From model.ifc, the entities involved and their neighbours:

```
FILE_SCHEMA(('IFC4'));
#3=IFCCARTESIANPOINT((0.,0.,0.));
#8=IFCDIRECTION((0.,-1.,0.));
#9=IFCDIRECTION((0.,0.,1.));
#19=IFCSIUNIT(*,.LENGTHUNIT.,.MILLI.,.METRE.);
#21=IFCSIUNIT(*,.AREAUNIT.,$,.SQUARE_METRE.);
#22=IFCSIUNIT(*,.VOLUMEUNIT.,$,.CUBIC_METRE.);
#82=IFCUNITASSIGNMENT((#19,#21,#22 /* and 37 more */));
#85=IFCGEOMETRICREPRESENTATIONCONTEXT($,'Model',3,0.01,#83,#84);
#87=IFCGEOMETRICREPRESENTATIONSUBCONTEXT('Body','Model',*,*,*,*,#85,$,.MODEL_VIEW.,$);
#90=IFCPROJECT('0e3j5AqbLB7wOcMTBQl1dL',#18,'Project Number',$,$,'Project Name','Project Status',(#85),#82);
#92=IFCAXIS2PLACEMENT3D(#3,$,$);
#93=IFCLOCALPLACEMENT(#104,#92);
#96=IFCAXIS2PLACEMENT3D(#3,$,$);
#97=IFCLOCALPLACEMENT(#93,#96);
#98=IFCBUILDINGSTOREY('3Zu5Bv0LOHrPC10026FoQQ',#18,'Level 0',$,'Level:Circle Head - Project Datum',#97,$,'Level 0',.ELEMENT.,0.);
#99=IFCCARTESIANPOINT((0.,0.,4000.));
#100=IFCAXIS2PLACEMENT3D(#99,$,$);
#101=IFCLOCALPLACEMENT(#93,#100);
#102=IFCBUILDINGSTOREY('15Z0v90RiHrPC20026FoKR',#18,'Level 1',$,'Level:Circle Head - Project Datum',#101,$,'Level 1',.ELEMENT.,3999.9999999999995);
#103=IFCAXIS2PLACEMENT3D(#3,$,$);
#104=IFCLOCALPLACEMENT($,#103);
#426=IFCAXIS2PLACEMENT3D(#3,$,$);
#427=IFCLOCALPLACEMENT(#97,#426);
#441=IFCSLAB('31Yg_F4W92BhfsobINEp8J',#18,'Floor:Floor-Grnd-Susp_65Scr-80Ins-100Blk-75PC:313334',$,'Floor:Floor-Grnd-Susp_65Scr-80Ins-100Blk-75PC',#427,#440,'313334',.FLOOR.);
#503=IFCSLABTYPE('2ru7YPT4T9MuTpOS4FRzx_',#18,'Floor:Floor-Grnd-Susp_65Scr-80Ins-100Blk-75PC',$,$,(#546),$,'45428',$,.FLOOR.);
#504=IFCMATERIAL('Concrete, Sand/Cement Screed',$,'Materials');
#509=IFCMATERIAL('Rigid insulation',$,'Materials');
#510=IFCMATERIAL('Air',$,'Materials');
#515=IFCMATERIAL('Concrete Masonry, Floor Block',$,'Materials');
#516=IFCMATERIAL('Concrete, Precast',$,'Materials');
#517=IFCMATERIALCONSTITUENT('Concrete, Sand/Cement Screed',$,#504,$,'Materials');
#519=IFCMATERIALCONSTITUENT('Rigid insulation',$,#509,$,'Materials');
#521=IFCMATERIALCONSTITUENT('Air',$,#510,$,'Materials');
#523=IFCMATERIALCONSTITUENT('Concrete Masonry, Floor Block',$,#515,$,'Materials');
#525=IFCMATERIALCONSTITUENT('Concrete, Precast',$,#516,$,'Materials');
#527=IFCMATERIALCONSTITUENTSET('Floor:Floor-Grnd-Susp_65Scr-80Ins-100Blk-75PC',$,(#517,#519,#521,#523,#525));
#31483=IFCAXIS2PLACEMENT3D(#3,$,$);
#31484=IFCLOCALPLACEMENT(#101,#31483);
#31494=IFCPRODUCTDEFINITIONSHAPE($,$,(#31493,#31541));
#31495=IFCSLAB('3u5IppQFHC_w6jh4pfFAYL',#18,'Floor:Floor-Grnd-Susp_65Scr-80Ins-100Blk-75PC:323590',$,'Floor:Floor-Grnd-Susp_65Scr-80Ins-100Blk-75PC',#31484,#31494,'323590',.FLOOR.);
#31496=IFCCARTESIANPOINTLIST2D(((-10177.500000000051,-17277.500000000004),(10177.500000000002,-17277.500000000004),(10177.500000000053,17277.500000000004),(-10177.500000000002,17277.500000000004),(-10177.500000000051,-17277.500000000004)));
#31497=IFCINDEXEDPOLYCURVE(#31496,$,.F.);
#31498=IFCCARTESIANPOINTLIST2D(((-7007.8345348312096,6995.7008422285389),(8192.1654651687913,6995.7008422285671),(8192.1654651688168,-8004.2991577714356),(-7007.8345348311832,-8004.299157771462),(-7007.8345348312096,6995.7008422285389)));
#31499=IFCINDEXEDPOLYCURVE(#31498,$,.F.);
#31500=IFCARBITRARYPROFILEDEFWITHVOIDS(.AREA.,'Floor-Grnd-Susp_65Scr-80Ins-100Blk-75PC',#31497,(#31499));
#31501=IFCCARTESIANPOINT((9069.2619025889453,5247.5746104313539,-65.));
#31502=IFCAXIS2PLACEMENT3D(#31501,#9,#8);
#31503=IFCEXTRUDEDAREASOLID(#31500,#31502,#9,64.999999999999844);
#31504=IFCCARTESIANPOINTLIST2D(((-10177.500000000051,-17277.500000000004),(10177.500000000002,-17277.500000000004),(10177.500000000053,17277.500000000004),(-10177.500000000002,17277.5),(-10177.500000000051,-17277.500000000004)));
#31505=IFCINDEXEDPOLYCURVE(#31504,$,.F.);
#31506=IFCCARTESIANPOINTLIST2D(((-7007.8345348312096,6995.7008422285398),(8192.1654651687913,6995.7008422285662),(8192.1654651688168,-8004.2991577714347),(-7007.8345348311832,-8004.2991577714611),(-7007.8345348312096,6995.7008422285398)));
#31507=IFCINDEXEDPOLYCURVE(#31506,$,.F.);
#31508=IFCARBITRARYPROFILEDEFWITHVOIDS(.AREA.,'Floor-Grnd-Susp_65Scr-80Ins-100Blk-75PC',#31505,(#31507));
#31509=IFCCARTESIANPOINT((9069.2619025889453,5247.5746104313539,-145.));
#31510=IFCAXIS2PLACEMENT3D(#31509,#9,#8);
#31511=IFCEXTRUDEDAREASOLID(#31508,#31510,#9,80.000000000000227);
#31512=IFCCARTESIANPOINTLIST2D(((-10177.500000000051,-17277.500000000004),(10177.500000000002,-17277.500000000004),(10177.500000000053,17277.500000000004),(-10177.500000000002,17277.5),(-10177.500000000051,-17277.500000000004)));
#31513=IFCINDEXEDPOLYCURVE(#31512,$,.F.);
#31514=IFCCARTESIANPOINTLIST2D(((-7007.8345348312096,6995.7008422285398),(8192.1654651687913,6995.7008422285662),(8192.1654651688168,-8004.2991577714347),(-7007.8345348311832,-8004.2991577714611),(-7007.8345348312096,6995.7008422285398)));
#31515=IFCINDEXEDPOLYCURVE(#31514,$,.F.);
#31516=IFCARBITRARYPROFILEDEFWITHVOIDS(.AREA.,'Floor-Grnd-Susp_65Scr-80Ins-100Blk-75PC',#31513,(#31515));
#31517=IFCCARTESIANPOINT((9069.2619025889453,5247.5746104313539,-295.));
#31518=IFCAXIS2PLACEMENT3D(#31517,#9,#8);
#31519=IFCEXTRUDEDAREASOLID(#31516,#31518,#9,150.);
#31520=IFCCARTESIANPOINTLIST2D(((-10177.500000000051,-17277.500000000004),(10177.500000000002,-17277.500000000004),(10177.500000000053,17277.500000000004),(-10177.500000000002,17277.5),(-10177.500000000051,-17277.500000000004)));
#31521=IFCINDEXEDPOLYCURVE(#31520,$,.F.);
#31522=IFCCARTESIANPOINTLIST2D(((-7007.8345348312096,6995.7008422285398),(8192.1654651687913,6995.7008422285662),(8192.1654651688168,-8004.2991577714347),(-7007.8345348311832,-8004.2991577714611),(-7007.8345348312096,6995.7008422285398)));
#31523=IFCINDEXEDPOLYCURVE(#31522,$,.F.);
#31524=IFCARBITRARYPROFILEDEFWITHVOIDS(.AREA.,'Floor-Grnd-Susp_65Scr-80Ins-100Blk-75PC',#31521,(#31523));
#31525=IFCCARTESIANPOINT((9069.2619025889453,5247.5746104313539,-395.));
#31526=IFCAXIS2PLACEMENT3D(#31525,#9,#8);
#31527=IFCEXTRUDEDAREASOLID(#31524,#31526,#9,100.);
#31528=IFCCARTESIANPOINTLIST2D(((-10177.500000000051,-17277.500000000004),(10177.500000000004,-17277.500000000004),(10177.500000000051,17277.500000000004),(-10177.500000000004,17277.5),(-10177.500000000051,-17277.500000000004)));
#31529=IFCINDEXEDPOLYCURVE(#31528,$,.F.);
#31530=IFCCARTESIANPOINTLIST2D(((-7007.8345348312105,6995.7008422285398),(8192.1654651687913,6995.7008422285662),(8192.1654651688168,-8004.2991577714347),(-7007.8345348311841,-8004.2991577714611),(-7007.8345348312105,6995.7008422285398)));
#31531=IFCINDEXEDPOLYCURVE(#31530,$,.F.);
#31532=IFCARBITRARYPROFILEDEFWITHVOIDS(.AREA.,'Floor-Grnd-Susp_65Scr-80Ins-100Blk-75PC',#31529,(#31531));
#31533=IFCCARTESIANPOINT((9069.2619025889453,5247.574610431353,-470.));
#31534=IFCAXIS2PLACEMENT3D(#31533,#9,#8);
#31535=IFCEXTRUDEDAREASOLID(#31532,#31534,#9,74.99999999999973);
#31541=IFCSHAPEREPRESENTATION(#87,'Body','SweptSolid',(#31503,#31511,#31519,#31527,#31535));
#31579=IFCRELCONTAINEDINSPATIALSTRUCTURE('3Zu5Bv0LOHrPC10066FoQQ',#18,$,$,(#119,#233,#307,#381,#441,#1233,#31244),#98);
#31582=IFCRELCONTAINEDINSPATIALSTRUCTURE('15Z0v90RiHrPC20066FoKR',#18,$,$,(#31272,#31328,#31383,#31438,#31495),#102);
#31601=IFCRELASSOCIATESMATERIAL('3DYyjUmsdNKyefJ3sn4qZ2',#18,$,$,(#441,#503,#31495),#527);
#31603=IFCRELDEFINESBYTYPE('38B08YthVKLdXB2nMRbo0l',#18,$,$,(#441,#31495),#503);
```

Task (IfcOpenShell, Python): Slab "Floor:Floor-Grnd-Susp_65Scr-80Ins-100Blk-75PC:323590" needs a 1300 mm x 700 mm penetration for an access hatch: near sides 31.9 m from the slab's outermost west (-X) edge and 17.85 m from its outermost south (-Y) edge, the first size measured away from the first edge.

```python
import numpy as np
import ifcopenshell
import ifcopenshell.api.feature
import ifcopenshell.api.geometry
import ifcopenshell.api.root
import ifcopenshell.geom
import ifcopenshell.util.placement
import ifcopenshell.util.representation
import ifcopenshell.util.shape
import ifcopenshell.util.unit

model = ifcopenshell.open("model.ifc")
unit_scale = ifcopenshell.util.unit.calculate_unit_scale(model)
settings = ifcopenshell.geom.settings()


def volume(element):
    """Net volume in cubic metres, openings subtracted."""
    shape = ifcopenshell.geom.create_shape(settings, element)
    return ifcopenshell.util.shape.get_volume(shape.geometry)


slab = model.by_guid("3u5IppQFHC_w6jh4pfFAYL")
before = volume(slab)

# Extent in the slab's own axes, in metres. The edges named are its -X and -Y sides.
slab_shape = ifcopenshell.geom.create_shape(settings, slab)
vertices = ifcopenshell.util.shape.get_vertices(slab_shape.geometry)
x_min, y_min, bottom = vertices.min(axis=0)
top = vertices[:, 2].max()

opening = ifcopenshell.api.root.create_entity(model, ifc_class="IfcOpeningElement", name="Access hatch opening", predefined_type="OPENING")
context = ifcopenshell.util.representation.get_context(model, "Model", "Body", "MODEL_VIEW")
width, depth = 1.3, 0.7
outline = [(0.0, 0.0), (width, 0.0), (width, depth), (0.0, depth), (0.0, 0.0)]
# Overshoot both faces by 50 mm so the cut is clean.
shape = ifcopenshell.api.geometry.add_slab_representation(
    model, context=context, depth=top - bottom + 0.1, polyline=outline
)
ifcopenshell.api.geometry.assign_representation(model, product=opening, representation=shape)

matrix = ifcopenshell.util.placement.get_local_placement(slab.ObjectPlacement)
matrix[:, 3] = matrix @ np.append(np.array([x_min + 31.9, y_min + 17.85, bottom - 0.05]) / unit_scale, 1.0)
ifcopenshell.api.geometry.edit_object_placement(model, product=opening, matrix=matrix, is_si=False)
ifcopenshell.api.feature.add_feature(model, feature=opening, element=slab)

after = volume(slab)

print(f"slab volume {before:.3f} -> {after:.3f} m3")

model.write("model_edited.ifc")
```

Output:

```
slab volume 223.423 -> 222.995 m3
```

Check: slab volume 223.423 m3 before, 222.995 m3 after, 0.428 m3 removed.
